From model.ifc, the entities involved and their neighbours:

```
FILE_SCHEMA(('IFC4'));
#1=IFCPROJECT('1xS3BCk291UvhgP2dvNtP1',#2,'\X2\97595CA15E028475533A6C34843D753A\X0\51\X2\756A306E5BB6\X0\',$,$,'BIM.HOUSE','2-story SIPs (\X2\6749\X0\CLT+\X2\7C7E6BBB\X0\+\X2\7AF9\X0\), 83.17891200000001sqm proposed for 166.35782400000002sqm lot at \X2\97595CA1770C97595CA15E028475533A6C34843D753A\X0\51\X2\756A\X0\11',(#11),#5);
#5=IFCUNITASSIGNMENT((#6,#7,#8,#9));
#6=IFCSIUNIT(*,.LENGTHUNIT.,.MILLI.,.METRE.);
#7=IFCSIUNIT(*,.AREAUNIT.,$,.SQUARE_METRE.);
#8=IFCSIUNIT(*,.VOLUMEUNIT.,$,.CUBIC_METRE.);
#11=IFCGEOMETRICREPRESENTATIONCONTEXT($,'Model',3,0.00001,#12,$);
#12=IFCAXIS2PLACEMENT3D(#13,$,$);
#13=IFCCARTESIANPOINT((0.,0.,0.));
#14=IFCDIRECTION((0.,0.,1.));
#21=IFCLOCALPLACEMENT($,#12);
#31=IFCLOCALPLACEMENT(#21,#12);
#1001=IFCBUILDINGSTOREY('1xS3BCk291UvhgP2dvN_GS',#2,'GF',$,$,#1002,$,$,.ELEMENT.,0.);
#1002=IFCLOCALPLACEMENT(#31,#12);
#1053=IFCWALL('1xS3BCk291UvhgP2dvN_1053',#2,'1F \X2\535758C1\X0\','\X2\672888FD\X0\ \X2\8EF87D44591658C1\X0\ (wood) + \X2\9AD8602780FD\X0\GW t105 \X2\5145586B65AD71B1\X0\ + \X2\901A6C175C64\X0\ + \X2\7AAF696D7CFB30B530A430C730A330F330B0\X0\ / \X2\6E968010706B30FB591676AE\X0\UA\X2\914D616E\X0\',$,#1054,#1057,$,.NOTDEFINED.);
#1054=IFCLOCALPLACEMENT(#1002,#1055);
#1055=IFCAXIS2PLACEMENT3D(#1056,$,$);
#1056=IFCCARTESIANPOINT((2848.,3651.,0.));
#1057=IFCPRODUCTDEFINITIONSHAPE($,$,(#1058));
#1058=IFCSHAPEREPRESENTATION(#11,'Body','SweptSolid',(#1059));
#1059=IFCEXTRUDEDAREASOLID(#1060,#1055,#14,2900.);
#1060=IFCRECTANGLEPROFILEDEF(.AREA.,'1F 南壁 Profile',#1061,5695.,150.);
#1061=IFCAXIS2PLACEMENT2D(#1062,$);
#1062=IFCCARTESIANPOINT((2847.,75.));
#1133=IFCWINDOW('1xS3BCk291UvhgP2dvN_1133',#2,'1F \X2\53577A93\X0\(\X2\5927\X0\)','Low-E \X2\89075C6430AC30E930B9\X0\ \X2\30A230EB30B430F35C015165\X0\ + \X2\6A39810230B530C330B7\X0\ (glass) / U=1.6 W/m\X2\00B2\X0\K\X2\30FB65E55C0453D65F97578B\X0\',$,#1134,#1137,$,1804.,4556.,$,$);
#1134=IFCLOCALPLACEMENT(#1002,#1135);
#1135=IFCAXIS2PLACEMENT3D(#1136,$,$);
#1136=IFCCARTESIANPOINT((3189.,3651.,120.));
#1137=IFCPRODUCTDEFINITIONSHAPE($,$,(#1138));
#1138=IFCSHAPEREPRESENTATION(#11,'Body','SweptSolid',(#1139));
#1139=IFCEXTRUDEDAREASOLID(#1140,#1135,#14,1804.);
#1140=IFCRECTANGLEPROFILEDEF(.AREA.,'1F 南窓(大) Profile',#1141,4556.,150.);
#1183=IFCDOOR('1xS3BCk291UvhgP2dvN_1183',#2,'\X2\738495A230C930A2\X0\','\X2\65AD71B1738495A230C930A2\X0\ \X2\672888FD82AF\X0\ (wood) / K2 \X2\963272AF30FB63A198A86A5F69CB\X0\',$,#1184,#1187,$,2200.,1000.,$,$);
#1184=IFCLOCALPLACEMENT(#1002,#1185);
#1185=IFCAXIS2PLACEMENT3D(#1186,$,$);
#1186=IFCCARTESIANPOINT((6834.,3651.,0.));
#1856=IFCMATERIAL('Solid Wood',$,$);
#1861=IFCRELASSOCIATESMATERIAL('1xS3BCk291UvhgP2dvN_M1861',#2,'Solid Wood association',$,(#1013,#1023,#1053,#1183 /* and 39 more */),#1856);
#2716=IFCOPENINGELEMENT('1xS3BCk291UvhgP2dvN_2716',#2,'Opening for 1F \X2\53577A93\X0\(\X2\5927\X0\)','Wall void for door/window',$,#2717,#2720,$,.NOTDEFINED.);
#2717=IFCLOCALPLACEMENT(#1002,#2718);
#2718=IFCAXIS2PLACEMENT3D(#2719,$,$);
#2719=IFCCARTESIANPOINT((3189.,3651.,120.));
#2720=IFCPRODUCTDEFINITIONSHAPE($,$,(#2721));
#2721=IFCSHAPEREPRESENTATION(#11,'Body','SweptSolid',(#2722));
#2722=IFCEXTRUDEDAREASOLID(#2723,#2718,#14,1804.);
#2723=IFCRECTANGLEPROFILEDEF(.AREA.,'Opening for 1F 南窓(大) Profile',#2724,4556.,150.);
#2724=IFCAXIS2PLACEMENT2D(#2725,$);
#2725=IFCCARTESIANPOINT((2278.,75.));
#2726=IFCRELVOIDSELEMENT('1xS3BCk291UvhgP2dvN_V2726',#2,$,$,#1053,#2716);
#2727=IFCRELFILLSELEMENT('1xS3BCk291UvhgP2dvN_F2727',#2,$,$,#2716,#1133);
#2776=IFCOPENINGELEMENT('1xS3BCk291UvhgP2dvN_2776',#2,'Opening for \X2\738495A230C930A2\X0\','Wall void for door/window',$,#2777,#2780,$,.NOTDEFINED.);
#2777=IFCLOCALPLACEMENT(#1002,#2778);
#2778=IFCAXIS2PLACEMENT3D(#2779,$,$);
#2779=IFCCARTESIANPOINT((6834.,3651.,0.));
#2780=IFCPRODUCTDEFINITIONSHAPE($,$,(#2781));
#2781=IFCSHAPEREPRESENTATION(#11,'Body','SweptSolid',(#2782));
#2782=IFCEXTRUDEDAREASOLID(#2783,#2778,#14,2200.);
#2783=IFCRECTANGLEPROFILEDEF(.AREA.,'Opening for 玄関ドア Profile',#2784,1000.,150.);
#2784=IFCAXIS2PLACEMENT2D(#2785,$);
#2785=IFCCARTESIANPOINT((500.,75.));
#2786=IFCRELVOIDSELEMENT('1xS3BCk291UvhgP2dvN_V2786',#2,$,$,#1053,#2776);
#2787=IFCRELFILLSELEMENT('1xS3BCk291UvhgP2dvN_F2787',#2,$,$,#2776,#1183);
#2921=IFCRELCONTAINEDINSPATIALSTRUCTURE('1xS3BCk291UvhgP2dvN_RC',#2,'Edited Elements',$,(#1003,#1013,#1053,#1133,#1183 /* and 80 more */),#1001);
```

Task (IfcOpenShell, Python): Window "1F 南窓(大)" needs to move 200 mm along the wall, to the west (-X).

```python
import ifcopenshell
import ifcopenshell.api.geometry
import ifcopenshell.util.placement

model = ifcopenshell.open("model.ifc")

window = model.by_guid("1xS3BCk291UvhgP2dvN_1133")
opening = window.FillsVoids[0].RelatingOpeningElement
wall = opening.VoidsElements[0].RelatingBuildingElement

wall_matrix = ifcopenshell.util.placement.get_local_placement(wall.ObjectPlacement)
shift = wall_matrix[:3, 0] * -200.0
before = ifcopenshell.util.placement.get_local_placement(window.ObjectPlacement)[:3, 3].copy()

# The window is not placed relative to its opening, so move both.
for product in (opening, window):
    matrix = ifcopenshell.util.placement.get_local_placement(product.ObjectPlacement)
    matrix[:3, 3] += shift
    ifcopenshell.api.geometry.edit_object_placement(model, product=product, matrix=matrix, is_si=False)

after = ifcopenshell.util.placement.get_local_placement(window.ObjectPlacement)[:3, 3]
print("window moved by", (after - before).round(3) + 0.0)

model.write("model_rev.ifc")
```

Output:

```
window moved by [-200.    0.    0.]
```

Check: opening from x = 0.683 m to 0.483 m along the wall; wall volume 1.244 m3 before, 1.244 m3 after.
